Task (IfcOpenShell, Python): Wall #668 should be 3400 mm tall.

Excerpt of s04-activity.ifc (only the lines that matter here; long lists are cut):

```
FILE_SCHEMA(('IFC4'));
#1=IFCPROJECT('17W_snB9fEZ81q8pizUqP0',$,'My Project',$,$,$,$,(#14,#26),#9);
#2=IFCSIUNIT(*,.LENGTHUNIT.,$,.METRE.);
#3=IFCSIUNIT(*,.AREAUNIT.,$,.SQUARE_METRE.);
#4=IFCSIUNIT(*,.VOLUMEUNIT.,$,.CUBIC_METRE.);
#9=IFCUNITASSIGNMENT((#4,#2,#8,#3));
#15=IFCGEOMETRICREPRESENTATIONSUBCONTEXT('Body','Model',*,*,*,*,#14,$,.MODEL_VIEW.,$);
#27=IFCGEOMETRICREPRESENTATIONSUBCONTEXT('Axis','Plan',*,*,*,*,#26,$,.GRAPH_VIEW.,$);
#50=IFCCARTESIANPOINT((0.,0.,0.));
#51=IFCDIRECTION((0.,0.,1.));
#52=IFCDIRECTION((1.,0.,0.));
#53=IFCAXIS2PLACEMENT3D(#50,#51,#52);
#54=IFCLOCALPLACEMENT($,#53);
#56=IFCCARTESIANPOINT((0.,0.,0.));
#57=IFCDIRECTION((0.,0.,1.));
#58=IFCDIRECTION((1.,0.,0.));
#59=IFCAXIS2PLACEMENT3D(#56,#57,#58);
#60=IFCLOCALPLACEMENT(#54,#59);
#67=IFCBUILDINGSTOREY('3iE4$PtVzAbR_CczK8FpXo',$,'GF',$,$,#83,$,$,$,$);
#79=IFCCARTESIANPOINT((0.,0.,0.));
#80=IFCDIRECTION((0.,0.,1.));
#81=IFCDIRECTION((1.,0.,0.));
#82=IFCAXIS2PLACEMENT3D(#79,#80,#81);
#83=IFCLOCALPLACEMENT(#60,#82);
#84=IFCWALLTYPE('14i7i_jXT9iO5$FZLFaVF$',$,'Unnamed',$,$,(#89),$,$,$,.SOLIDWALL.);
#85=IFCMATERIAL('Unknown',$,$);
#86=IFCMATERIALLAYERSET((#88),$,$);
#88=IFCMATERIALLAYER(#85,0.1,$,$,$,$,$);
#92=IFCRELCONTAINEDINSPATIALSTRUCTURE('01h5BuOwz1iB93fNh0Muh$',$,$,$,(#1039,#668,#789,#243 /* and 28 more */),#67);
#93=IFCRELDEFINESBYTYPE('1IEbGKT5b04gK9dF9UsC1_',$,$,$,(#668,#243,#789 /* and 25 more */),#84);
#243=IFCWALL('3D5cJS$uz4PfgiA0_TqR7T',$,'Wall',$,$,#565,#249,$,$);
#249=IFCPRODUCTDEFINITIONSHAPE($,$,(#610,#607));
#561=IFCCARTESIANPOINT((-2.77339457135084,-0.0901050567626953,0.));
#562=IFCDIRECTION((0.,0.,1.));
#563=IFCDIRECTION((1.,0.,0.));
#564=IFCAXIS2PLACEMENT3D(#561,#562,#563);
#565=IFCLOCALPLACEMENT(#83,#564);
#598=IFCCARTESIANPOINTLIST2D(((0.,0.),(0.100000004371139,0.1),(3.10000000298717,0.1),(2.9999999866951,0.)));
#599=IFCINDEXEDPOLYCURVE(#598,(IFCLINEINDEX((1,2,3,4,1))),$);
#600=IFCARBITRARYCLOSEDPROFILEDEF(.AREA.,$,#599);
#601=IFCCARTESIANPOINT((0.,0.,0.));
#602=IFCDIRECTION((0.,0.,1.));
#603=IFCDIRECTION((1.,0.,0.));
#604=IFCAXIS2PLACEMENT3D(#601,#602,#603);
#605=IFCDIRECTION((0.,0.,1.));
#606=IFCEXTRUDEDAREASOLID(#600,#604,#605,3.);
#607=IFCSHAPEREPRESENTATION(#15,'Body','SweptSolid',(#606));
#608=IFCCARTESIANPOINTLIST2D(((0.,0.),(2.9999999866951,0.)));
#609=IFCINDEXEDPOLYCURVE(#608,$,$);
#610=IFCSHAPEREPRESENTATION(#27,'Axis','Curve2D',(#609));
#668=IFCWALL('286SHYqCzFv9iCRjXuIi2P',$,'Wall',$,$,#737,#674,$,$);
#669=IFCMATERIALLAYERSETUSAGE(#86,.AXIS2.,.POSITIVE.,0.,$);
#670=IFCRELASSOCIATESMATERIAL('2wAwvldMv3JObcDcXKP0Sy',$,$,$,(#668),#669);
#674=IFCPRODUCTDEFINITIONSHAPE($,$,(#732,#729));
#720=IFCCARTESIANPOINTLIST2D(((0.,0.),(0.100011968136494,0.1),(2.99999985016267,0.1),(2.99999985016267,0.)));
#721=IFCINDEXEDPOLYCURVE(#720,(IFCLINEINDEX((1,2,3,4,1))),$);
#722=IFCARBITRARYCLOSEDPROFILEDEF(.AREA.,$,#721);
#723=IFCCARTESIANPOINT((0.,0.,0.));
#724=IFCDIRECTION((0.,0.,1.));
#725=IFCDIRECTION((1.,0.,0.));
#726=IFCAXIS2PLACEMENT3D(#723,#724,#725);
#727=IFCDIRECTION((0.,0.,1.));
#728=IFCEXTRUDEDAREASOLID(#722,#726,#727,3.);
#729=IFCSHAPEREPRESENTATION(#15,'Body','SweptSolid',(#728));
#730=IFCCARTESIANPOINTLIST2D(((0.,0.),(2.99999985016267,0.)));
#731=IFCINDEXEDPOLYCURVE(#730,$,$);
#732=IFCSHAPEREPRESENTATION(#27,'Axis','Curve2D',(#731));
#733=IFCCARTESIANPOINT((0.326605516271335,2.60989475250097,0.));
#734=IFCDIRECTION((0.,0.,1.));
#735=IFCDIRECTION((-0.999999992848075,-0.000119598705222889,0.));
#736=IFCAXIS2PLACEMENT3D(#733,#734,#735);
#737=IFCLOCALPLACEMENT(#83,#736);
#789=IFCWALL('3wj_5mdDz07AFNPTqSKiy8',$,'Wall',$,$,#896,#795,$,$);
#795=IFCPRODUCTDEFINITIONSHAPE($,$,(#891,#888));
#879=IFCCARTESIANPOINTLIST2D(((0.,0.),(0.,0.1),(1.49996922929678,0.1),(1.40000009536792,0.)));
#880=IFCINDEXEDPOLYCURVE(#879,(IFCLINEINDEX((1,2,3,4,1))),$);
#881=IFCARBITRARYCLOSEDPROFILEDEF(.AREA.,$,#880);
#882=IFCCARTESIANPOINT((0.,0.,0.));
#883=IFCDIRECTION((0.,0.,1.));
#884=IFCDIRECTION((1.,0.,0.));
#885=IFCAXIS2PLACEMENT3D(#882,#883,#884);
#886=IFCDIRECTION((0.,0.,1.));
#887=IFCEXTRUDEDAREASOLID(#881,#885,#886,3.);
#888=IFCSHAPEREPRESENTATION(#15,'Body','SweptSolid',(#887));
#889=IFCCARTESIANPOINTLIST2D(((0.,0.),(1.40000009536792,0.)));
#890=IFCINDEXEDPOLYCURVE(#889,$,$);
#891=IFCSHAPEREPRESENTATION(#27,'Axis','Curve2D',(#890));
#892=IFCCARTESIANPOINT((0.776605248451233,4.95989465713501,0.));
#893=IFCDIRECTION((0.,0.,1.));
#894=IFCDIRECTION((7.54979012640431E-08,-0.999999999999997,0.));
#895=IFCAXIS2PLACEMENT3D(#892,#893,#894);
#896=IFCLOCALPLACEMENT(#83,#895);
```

```python
import ifcopenshell
import ifcopenshell.geom
import ifcopenshell.util.representation
import ifcopenshell.util.shape
import ifcopenshell.util.unit

model = ifcopenshell.open("s04-activity.ifc")
unit_scale = ifcopenshell.util.unit.calculate_unit_scale(model)
settings = ifcopenshell.geom.settings()


def volume(element):
    """Net volume in cubic metres, openings subtracted."""
    shape = ifcopenshell.geom.create_shape(settings, element)
    return ifcopenshell.util.shape.get_volume(shape.geometry)


wall = model.by_guid("286SHYqCzFv9iCRjXuIi2P")
before = volume(wall)

body = ifcopenshell.util.representation.get_representation(wall, "Model", "Body")
solid = body.Items[0]
old_height = solid.Depth
solid.Depth = 3.4 / unit_scale
after = volume(wall)

print(f"height {old_height:g} -> {solid.Depth:g}, volume {before:.3f} -> {after:.3f} m3")

model.write("s04-activity_rev.ifc")
```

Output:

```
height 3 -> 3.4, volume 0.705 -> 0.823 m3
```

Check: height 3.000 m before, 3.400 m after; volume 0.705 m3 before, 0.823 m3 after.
